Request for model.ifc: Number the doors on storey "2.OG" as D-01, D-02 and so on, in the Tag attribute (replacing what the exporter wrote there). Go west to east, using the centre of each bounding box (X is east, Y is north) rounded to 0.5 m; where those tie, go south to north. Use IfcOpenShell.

First a look at what the model holds.

```python
import ifcopenshell
import ifcopenshell.util.element
import ifcopenshell.util.placement

model = ifcopenshell.open("model.ifc")
print(model.schema)
storey = next(s for s in model.by_type("IfcBuildingStorey") if s.Name == "2.OG")
doors = [e for e in ifcopenshell.util.element.get_decomposition(storey) if e.is_a("IfcDoor")]
for e in sorted(doors, key=lambda e: e.id()):
    origin = ifcopenshell.util.placement.get_local_placement(e.ObjectPlacement)[:3, 3]
    print(e.id(), e.Tag, e.Name, origin.round(2) + 0.0, sep=" | ")
```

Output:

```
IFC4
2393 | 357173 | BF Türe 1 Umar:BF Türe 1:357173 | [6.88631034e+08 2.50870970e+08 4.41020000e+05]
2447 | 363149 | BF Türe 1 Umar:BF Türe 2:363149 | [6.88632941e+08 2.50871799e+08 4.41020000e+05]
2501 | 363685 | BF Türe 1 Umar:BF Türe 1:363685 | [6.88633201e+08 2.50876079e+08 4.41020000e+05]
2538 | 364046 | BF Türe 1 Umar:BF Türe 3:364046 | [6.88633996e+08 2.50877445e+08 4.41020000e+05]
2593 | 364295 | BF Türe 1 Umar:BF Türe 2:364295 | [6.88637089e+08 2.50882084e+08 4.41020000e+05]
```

```python
import ifcopenshell
import ifcopenshell.geom
import ifcopenshell.util.element
import ifcopenshell.util.shape

model = ifcopenshell.open("model.ifc")
settings = ifcopenshell.geom.settings()
settings.set("use-world-coords", True)


def centre(element):
    shape = ifcopenshell.geom.create_shape(settings, element)
    return ifcopenshell.util.shape.get_bbox_centroid(shape.geometry)


storey = next(s for s in model.by_type("IfcBuildingStorey") if s.Name == "2.OG")
doors = [e for e in ifcopenshell.util.element.get_decomposition(storey) if e.is_a("IfcDoor")]

# Insertion points can sit at a corner or the storey origin, so sort by the geometry (in metres).
centres = {e: centre(e) for e in doors}
doors.sort(key=lambda e: (round(centres[e][0] / 0.5), centres[e][1]))

for i, e in enumerate(doors, start=1):
    number = f"D-{i:02d}"
    e.Tag = number
    print(e.id(), number)

model.write("model_edited.ifc")
```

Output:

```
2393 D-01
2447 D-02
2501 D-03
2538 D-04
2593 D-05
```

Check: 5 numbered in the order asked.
